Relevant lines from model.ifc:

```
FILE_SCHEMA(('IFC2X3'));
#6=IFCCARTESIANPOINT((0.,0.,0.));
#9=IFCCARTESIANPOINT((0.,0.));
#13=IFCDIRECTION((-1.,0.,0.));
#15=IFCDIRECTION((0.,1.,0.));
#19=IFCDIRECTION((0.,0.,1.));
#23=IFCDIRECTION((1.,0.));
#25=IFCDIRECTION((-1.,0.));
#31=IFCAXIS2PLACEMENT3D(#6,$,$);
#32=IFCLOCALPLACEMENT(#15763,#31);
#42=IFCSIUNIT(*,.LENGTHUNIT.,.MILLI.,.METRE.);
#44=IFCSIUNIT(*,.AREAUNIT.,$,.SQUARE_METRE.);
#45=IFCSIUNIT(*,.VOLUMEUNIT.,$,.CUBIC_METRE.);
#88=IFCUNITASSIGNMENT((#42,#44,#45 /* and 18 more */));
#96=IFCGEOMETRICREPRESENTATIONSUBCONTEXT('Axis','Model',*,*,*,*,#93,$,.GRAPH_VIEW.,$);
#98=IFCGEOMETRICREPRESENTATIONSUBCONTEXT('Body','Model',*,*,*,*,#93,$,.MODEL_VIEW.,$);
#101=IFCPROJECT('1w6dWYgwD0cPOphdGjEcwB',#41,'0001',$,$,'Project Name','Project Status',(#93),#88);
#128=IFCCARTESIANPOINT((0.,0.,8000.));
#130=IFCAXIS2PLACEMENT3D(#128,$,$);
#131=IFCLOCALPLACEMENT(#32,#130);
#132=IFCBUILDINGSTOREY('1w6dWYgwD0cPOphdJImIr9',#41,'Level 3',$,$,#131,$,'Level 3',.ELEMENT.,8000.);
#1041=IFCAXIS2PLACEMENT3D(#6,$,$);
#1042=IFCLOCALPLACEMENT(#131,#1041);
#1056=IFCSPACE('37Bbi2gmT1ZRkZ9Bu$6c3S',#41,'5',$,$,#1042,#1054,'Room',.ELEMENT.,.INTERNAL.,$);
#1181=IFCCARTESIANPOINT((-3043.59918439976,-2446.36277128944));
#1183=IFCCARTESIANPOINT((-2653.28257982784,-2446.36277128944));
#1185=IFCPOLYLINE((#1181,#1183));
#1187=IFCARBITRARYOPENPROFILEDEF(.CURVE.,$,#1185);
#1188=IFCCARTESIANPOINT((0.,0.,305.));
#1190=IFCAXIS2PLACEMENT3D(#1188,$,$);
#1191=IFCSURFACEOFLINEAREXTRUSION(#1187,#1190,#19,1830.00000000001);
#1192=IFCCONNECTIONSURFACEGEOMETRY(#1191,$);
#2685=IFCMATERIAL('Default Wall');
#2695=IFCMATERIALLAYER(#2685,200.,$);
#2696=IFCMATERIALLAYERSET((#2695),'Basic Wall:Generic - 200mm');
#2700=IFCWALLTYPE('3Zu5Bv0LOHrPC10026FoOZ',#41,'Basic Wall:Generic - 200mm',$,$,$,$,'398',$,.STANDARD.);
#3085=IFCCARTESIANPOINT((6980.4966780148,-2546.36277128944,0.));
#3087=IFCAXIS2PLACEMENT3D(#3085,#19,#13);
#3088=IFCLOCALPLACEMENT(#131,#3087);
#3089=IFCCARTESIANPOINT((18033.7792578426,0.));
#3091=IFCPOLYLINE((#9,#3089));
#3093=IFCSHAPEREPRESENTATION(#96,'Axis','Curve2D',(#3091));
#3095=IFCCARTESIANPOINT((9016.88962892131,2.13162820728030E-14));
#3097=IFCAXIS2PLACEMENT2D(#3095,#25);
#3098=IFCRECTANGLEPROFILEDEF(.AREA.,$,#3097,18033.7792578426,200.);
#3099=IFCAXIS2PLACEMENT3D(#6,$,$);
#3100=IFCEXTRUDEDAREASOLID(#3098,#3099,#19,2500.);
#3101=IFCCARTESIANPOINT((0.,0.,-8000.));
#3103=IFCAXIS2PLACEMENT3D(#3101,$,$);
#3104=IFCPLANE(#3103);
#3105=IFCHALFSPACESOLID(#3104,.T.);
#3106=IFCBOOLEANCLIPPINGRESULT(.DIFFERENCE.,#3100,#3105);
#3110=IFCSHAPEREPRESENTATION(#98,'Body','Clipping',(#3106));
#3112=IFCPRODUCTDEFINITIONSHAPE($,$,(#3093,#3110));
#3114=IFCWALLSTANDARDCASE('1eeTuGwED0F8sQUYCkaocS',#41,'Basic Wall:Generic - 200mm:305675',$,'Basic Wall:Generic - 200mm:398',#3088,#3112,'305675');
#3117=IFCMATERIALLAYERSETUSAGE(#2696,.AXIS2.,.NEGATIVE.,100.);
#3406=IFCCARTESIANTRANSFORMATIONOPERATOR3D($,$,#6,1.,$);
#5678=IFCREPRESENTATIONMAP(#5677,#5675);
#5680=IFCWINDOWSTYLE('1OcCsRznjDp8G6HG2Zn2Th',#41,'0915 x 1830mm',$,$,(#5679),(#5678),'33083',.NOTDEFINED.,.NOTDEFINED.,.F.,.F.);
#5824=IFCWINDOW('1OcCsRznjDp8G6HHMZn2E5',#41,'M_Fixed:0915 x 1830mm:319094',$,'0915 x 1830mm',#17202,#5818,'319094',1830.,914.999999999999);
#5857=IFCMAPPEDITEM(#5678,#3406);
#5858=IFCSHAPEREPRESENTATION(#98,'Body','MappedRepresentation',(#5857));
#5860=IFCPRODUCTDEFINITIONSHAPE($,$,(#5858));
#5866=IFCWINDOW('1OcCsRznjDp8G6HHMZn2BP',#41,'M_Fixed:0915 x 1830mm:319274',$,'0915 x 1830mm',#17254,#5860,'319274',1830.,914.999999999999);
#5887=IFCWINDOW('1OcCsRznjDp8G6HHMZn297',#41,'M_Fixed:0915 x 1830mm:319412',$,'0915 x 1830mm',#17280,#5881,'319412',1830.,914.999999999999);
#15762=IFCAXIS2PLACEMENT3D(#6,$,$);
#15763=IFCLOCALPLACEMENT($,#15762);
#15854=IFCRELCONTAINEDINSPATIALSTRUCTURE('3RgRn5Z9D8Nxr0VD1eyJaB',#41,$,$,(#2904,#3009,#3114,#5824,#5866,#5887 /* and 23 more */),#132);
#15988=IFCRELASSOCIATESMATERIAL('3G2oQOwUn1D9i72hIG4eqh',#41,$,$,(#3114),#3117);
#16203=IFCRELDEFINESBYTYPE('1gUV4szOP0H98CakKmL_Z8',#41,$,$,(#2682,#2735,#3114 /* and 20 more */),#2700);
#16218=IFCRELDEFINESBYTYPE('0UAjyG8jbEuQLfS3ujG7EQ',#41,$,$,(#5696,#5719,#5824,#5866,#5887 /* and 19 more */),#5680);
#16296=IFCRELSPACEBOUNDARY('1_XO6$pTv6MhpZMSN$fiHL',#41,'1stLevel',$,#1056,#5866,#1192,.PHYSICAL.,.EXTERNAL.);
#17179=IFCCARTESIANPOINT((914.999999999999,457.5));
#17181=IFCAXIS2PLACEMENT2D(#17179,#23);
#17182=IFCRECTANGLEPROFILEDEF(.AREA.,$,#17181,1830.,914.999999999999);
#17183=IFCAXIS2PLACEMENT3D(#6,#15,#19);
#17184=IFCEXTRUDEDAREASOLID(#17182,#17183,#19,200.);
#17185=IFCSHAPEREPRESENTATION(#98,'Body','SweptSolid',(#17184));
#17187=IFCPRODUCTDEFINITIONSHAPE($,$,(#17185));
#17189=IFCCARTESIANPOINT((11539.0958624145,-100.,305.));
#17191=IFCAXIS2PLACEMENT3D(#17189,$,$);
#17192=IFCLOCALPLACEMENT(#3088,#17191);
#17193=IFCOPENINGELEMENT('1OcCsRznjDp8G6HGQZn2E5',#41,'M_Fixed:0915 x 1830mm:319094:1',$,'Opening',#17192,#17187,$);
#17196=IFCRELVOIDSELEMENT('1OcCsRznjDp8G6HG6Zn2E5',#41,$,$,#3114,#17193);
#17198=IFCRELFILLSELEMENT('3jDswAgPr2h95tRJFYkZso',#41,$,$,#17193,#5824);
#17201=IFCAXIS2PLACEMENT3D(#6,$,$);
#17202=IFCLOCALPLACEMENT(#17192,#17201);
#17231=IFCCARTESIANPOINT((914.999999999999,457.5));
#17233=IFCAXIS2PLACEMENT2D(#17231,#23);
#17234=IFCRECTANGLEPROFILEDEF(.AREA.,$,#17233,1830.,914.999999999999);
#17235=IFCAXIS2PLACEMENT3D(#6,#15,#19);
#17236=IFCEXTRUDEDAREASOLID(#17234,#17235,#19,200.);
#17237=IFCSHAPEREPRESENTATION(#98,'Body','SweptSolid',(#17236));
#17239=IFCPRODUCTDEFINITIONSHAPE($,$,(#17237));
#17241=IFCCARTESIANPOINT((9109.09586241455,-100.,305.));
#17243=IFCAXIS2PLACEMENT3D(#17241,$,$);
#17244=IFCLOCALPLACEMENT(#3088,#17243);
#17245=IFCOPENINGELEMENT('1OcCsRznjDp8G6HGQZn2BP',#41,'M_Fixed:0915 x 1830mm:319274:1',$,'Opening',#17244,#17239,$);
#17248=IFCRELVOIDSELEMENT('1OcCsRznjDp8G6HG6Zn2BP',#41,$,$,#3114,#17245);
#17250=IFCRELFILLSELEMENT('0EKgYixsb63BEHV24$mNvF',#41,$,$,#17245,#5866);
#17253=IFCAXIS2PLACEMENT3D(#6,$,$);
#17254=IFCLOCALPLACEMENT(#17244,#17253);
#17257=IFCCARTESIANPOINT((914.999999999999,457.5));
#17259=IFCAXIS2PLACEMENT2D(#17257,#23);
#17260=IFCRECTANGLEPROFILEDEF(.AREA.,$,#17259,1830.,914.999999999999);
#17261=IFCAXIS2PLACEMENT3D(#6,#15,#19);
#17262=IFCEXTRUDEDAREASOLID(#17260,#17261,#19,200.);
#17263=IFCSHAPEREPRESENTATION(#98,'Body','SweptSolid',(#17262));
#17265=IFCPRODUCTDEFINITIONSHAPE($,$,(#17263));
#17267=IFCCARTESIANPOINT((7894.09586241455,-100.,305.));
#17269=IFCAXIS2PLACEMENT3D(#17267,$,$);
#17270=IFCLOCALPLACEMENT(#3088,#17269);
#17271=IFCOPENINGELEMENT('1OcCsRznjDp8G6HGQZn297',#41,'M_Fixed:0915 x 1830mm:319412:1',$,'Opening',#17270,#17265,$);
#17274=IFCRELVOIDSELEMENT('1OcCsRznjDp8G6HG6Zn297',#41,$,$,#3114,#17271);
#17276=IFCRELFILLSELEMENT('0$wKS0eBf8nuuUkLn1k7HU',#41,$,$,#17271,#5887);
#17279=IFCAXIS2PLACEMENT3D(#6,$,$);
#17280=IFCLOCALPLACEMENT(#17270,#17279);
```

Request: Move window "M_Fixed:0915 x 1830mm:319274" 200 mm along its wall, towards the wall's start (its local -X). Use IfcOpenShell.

```python
import numpy as np
import ifcopenshell
import ifcopenshell.api.geometry
import ifcopenshell.util.placement
import ifcopenshell.util.unit

model = ifcopenshell.open("model.ifc")
unit_scale = ifcopenshell.util.unit.calculate_unit_scale(model)

window = model.by_id(5866)
opening = window.FillsVoids[0].RelatingOpeningElement
wall = opening.VoidsElements[0].RelatingBuildingElement

wall_matrix = ifcopenshell.util.placement.get_local_placement(wall.ObjectPlacement)
shift = wall_matrix[:3, 0] * -0.2 / unit_scale
before = ifcopenshell.util.placement.get_local_placement(window.ObjectPlacement)[:3, 3].copy()

# The window is placed relative to its opening, so it follows when the opening moves.
matrix = ifcopenshell.util.placement.get_local_placement(opening.ObjectPlacement)
matrix[:3, 3] += shift
ifcopenshell.api.geometry.edit_object_placement(
    model, product=opening, matrix=matrix, is_si=False, should_transform_children=True
)

# Space boundary surfaces are stored in each space's coordinates; move them too.
for rel in window.ProvidesBoundaries:
    if not rel.ConnectionGeometry:
        continue
    surface = rel.ConnectionGeometry.SurfaceOnRelatingElement
    space_matrix = ifcopenshell.util.placement.get_local_placement(rel.RelatingSpace.ObjectPlacement)
    point = np.array(surface.Position.Location.Coordinates) + space_matrix[:3, :3].T @ shift
    surface.Position = model.createIfcAxis2Placement3D(
        model.createIfcCartesianPoint(point.tolist()), surface.Position.Axis, surface.Position.RefDirection
    )

after = ifcopenshell.util.placement.get_local_placement(window.ObjectPlacement)[:3, 3]
print("window moved by", (after - before).round(3) + 0.0)

model.write("model_updated.ifc")
```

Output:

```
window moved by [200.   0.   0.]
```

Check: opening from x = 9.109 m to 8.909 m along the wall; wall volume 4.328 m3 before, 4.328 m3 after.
